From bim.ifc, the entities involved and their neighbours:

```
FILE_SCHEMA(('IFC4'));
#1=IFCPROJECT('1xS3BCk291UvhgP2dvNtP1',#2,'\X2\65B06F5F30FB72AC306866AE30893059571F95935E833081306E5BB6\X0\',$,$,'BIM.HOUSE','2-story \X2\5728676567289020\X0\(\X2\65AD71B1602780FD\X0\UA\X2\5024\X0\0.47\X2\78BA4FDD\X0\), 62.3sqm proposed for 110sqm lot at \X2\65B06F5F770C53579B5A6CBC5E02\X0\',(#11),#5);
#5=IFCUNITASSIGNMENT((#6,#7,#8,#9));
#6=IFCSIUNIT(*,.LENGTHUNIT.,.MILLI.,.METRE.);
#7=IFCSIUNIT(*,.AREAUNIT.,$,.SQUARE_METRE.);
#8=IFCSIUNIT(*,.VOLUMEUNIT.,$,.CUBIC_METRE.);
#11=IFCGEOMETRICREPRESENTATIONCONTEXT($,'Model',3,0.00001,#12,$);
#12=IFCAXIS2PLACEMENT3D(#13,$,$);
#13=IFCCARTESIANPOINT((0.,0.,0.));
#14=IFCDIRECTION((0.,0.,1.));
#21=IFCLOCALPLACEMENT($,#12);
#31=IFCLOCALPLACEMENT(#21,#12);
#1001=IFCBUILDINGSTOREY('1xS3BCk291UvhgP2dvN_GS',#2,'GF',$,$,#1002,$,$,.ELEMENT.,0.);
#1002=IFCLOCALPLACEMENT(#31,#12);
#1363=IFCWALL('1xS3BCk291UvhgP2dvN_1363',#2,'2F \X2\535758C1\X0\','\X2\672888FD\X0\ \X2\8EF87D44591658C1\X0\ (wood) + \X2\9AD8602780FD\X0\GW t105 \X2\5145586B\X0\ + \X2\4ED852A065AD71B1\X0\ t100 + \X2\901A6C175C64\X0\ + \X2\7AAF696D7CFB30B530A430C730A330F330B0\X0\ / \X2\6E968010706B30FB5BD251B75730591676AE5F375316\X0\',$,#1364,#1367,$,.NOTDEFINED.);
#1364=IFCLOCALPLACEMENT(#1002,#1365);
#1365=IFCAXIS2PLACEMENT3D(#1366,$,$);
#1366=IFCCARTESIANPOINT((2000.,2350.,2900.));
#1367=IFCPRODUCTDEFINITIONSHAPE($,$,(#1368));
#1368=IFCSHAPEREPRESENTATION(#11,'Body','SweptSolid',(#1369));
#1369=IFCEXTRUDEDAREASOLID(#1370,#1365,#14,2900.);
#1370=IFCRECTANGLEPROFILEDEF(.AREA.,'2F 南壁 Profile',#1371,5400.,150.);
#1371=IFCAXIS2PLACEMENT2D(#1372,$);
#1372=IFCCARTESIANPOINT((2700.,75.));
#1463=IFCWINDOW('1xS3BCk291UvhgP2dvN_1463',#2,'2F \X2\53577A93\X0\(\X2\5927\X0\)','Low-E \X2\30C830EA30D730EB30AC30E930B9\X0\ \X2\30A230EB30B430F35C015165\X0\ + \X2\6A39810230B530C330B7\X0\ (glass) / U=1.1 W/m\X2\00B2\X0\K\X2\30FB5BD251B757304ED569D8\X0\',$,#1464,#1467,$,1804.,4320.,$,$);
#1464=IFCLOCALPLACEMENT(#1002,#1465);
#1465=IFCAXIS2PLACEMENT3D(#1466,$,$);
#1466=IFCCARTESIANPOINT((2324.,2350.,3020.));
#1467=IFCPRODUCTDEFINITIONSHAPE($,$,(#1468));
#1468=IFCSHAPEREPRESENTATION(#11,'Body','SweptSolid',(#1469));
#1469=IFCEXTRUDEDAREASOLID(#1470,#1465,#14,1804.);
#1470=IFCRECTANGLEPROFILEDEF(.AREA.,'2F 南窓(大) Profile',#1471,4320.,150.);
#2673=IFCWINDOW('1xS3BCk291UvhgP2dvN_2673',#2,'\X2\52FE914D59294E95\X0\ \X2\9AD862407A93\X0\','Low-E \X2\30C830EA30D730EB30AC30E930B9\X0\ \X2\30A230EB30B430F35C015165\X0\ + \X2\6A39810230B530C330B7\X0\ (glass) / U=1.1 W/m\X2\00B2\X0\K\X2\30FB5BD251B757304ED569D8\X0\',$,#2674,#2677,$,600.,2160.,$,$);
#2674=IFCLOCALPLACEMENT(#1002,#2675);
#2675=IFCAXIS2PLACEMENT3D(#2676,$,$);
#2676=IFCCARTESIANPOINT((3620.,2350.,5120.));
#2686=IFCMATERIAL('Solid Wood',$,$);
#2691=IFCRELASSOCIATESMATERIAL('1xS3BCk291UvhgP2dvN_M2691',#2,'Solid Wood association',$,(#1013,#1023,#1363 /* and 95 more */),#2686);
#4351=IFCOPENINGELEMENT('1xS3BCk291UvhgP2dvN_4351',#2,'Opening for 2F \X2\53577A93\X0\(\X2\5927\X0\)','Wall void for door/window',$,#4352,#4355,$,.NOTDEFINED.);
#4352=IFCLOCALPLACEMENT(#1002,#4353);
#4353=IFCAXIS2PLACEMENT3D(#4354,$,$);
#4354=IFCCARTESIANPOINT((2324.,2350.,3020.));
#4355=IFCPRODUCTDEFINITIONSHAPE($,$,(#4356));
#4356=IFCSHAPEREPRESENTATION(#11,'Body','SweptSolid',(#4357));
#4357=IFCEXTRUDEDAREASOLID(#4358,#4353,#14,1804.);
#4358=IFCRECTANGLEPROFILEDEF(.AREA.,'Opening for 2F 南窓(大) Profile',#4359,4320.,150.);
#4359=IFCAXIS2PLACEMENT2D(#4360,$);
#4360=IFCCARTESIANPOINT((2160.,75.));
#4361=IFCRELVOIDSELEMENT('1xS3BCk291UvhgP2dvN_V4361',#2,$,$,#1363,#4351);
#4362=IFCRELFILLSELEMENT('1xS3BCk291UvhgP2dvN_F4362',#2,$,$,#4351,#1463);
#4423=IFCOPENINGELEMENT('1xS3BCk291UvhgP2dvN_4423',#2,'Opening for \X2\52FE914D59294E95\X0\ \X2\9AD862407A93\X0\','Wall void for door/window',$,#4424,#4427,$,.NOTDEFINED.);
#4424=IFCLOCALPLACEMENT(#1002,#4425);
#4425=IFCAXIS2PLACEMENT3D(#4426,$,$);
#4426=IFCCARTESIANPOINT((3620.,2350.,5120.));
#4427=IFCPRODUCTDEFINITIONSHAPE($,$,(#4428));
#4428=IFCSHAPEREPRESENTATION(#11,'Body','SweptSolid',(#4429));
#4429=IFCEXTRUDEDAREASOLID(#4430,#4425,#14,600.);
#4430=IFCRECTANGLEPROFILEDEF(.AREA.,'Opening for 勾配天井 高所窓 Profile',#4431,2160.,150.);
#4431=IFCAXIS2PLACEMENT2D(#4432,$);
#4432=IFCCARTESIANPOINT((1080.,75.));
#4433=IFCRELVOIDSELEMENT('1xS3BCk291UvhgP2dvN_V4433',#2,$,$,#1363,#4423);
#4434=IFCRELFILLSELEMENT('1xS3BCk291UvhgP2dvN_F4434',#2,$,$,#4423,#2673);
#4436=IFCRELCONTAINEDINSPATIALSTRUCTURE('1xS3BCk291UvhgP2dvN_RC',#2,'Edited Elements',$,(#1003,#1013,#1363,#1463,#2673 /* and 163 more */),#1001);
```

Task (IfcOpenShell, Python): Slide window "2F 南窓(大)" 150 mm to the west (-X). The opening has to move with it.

```python
import ifcopenshell
import ifcopenshell.api.geometry
import ifcopenshell.util.placement
import ifcopenshell.util.unit

model = ifcopenshell.open("bim.ifc")
unit_scale = ifcopenshell.util.unit.calculate_unit_scale(model)

window = model.by_id(1463)
opening = window.FillsVoids[0].RelatingOpeningElement
wall = opening.VoidsElements[0].RelatingBuildingElement

wall_matrix = ifcopenshell.util.placement.get_local_placement(wall.ObjectPlacement)
shift = wall_matrix[:3, 0] * -0.15 / unit_scale
before = ifcopenshell.util.placement.get_local_placement(window.ObjectPlacement)[:3, 3].copy()

# The window is not placed relative to its opening, so move both.
for product in (opening, window):
    matrix = ifcopenshell.util.placement.get_local_placement(product.ObjectPlacement)
    matrix[:3, 3] += shift
    ifcopenshell.api.geometry.edit_object_placement(model, product=product, matrix=matrix, is_si=False)

after = ifcopenshell.util.placement.get_local_placement(window.ObjectPlacement)[:3, 3]
print("window moved by", (after - before).round(3) + 0.0)

model.write("bim_updated.ifc")
```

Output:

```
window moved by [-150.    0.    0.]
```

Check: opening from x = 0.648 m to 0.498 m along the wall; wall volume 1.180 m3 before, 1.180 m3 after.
